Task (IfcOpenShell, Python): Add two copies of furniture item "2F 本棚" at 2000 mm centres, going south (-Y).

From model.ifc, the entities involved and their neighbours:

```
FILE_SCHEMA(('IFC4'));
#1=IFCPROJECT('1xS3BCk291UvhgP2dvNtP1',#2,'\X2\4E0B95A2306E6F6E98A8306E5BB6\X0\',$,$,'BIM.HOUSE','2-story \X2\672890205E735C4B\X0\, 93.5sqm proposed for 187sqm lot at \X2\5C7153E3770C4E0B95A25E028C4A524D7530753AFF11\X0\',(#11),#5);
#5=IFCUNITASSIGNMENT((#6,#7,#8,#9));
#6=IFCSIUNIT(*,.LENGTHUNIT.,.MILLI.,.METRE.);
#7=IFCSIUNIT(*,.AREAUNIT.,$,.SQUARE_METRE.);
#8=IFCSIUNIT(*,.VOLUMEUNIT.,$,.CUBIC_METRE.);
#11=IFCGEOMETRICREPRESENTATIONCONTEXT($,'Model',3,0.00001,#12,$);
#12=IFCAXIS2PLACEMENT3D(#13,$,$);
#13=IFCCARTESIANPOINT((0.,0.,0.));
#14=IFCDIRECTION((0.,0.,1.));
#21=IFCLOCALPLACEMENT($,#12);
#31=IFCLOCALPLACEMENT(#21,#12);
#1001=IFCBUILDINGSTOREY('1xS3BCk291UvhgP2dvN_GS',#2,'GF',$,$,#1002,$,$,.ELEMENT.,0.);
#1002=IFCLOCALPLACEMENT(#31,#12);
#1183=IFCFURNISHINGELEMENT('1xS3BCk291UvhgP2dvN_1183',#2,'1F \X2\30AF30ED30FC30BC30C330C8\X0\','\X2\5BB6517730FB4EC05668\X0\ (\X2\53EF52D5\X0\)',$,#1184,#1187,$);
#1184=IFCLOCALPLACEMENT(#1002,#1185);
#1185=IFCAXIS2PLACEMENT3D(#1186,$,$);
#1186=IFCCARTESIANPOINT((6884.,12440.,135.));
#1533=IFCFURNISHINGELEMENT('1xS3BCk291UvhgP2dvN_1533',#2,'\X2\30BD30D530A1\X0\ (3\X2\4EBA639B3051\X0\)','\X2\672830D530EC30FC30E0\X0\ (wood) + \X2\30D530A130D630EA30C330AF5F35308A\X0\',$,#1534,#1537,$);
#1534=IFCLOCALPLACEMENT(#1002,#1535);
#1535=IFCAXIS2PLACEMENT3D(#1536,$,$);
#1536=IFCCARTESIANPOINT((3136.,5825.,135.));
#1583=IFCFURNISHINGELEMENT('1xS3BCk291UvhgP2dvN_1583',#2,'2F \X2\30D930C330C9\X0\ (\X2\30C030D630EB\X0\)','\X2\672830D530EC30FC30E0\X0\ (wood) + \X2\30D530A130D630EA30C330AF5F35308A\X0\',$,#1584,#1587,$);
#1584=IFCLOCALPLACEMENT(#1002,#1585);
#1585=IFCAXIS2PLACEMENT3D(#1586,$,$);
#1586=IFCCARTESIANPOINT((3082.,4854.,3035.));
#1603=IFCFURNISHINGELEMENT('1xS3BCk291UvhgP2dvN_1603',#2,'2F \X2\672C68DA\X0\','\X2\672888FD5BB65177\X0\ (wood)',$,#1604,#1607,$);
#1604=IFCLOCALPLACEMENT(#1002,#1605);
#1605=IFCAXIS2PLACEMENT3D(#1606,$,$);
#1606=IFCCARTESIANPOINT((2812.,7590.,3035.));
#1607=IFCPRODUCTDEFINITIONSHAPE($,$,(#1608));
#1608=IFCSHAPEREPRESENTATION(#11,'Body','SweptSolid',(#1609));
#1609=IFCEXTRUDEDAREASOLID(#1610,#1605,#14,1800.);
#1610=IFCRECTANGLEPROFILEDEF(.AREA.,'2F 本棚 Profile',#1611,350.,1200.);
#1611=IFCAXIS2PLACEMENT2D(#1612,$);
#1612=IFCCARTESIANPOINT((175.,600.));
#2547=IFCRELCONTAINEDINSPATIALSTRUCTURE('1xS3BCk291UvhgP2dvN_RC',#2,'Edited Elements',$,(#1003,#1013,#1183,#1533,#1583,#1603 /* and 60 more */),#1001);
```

```python
import numpy as np
import ifcopenshell
import ifcopenshell.api.geometry
import ifcopenshell.api.root
import ifcopenshell.util.element
import ifcopenshell.util.placement
import ifcopenshell.util.unit

model = ifcopenshell.open("model.ifc")
unit_scale = ifcopenshell.util.unit.calculate_unit_scale(model)


def reuse_history(source, copy):
    """copy_class also copies each property set's owner history, people and application; keep the originals."""
    for rel in copy.IsDefinedBy:
        if rel.is_a("IfcRelDefinesByProperties") and (history := rel.RelatingPropertyDefinition.OwnerHistory):
            rel.RelatingPropertyDefinition.OwnerHistory = source.OwnerHistory
            ifcopenshell.util.element.remove_deep2(model, history)


source = model.by_id(1603)
base = ifcopenshell.util.placement.get_local_placement(source.ObjectPlacement)
step = np.array([0.0, -1.0, 0.0]) * 2 / unit_scale

for i in range(1, 3):
    copy = ifcopenshell.api.root.copy_class(model, product=source)
    copy.Representation = ifcopenshell.util.element.copy_deep(
        model, source.Representation, exclude=["IfcGeometricRepresentationContext", "IfcRepresentationMap"]
    )
    reuse_history(source, copy)
    matrix = base.copy()
    matrix[:3, 3] += i * step
    print("added at", matrix[:3, 3].round(3) + 0.0)
    ifcopenshell.api.geometry.edit_object_placement(model, product=copy, matrix=matrix, is_si=False)

model.write("model_updated.ifc")
```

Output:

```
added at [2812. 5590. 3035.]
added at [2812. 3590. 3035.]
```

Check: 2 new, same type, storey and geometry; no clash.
